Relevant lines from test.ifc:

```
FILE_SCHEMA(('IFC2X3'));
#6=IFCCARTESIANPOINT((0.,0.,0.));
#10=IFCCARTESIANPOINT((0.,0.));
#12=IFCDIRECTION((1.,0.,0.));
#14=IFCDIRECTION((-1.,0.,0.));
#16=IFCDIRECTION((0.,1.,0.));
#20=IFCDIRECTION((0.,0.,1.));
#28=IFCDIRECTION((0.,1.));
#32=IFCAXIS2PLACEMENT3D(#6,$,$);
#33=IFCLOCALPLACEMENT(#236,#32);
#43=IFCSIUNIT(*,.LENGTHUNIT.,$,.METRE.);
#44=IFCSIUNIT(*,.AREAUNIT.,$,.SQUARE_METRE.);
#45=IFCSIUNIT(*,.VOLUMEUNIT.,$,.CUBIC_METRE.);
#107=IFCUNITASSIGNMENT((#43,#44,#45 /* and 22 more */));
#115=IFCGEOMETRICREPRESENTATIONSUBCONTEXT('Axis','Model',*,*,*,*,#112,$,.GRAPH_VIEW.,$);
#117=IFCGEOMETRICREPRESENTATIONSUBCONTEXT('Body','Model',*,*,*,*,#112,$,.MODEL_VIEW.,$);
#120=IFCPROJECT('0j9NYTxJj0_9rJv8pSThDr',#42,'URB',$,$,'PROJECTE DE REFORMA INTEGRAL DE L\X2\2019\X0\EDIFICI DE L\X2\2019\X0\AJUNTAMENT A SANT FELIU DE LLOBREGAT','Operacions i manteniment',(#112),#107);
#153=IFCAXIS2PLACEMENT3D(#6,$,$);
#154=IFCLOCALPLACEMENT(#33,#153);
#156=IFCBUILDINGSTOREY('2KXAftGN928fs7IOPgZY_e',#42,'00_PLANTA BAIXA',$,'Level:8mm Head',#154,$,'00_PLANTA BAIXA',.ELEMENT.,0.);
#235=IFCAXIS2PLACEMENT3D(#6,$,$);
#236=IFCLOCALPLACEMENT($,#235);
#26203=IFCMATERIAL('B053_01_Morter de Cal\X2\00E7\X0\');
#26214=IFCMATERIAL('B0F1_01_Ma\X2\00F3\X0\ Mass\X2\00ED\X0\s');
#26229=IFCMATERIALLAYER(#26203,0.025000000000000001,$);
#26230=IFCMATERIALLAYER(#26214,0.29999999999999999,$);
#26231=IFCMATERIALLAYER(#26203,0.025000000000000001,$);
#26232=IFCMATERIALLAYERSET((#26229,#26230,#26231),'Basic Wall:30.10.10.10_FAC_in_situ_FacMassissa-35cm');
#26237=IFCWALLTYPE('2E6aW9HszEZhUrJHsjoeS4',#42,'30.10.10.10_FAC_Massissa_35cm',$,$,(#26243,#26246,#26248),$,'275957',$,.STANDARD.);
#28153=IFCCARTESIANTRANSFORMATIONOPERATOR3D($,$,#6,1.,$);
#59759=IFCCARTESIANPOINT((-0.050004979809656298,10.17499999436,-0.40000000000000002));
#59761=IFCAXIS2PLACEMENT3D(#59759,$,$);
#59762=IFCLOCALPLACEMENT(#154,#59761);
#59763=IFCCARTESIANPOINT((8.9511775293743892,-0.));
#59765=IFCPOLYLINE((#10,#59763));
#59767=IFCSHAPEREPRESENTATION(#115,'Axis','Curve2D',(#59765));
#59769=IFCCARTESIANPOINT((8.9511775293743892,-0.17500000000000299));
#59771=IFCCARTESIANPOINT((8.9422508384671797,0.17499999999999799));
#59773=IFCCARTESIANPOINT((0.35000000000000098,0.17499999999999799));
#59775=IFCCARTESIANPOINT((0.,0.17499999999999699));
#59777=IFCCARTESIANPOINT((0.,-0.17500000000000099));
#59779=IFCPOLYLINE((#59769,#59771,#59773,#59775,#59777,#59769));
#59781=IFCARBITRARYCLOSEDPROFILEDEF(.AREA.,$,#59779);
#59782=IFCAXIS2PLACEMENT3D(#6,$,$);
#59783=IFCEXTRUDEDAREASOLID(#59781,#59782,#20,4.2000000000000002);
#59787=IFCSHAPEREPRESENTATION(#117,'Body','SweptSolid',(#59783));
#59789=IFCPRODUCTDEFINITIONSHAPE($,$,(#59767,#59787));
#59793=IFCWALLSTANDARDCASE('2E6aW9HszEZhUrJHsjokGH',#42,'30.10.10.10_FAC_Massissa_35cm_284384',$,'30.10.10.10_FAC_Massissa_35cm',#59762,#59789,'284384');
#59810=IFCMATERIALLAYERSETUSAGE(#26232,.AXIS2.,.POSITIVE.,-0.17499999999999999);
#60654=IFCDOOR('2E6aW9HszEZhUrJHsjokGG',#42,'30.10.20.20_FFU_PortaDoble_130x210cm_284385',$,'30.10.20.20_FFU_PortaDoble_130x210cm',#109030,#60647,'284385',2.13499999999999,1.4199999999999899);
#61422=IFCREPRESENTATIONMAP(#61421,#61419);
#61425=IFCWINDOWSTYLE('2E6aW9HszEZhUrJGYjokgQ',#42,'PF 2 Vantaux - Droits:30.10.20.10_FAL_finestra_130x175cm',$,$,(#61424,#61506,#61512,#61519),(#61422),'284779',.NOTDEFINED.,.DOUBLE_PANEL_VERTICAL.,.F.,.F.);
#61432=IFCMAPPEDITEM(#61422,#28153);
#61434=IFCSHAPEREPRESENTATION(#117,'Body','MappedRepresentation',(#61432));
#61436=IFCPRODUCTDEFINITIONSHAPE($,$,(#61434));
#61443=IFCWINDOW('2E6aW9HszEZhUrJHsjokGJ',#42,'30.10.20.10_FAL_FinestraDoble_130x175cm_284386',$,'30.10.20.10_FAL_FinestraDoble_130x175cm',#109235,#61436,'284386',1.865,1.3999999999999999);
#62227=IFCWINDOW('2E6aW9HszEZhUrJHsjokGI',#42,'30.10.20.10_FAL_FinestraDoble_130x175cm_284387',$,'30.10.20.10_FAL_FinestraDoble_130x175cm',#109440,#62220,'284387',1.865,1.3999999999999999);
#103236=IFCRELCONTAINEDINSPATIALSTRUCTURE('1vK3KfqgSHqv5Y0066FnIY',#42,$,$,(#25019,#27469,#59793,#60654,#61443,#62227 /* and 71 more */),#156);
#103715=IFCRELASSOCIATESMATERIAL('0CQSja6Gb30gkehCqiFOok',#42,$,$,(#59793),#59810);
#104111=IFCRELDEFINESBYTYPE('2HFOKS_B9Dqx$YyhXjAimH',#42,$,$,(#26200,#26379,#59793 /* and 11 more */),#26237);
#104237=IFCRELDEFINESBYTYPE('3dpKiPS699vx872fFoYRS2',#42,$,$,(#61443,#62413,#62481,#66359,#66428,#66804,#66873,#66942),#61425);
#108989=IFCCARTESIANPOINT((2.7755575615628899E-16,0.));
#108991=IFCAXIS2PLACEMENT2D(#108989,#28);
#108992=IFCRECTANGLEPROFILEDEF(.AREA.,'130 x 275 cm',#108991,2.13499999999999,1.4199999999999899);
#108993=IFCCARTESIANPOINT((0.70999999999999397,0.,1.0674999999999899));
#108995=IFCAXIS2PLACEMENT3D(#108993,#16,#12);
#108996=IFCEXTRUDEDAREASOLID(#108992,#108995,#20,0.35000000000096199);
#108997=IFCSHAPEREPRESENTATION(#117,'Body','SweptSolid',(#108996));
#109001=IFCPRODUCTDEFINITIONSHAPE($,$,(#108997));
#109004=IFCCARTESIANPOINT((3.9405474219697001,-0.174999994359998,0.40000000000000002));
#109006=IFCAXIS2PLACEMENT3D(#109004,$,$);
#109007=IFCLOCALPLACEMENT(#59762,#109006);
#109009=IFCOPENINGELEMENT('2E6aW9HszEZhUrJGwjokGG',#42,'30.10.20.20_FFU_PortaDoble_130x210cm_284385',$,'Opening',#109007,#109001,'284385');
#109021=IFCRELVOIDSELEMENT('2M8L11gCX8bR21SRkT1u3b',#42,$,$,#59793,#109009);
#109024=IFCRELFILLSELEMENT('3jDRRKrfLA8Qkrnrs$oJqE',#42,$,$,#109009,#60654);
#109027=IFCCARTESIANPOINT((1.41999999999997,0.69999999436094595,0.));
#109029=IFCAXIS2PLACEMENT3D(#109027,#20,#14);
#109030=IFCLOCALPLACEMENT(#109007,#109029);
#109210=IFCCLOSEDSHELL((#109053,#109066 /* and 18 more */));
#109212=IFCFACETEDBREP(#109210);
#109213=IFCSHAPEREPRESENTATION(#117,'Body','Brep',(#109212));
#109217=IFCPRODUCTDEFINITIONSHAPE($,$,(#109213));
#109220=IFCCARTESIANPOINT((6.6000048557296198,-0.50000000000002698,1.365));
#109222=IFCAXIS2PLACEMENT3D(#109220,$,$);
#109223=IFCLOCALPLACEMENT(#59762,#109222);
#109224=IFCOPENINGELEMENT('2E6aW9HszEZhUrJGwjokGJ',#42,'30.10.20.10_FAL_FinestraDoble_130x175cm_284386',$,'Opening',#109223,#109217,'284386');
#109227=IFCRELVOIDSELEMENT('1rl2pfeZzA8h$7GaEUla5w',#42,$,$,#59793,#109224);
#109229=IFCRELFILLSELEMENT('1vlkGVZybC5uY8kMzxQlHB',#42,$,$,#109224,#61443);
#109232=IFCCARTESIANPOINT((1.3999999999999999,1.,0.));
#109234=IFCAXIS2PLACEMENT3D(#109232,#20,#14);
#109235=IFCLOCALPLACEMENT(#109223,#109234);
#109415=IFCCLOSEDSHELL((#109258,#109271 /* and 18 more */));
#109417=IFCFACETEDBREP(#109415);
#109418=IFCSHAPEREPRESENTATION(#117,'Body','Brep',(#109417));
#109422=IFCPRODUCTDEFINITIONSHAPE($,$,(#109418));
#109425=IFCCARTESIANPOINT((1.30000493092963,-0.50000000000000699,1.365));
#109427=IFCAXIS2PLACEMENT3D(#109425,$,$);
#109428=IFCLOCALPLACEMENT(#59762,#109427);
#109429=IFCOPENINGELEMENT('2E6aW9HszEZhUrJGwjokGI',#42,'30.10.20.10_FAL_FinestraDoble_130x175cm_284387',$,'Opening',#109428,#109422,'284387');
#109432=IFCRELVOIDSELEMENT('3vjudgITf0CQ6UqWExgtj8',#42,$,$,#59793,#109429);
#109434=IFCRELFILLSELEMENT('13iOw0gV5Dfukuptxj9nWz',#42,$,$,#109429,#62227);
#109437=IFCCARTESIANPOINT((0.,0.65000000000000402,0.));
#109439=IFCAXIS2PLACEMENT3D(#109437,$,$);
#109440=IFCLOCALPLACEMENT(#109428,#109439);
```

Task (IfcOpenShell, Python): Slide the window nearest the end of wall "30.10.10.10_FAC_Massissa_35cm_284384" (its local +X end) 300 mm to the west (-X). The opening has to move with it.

```python
import ifcopenshell
import ifcopenshell.api.geometry
import ifcopenshell.util.placement

model = ifcopenshell.open("test.ifc")

window = model.by_guid("2E6aW9HszEZhUrJHsjokGJ")
opening = window.FillsVoids[0].RelatingOpeningElement
wall = opening.VoidsElements[0].RelatingBuildingElement

wall_matrix = ifcopenshell.util.placement.get_local_placement(wall.ObjectPlacement)
shift = wall_matrix[:3, 0] * -0.3
before = ifcopenshell.util.placement.get_local_placement(window.ObjectPlacement)[:3, 3].copy()

# The window is placed relative to its opening, so it follows when the opening moves.
matrix = ifcopenshell.util.placement.get_local_placement(opening.ObjectPlacement)
matrix[:3, 3] += shift
ifcopenshell.api.geometry.edit_object_placement(
    model, product=opening, matrix=matrix, is_si=False, should_transform_children=True
)

after = ifcopenshell.util.placement.get_local_placement(window.ObjectPlacement)[:3, 3]
print("window moved by", (after - before).round(3) + 0.0)

model.write("test_rev.ifc")
```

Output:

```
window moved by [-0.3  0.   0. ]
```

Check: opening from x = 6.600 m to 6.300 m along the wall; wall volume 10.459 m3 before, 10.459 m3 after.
